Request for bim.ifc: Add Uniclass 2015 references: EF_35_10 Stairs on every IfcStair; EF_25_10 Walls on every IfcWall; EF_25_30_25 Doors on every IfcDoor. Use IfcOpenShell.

First a look at what the model holds.

```python
import ifcopenshell

model = ifcopenshell.open("bim.ifc")
print(model.schema)
print("classifications:", [c.Name for c in model.by_type("IfcClassification")])
for ifc_class in ("IfcDoor", "IfcRoof", "IfcStair", "IfcWall", "IfcWindow"):
    print(ifc_class, len(model.by_type(ifc_class)))
```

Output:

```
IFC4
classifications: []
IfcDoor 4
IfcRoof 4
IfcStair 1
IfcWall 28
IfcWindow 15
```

```python
import ifcopenshell
import ifcopenshell.api.classification

model = ifcopenshell.open("bim.ifc")

system = ifcopenshell.api.classification.add_classification(model, classification="Uniclass 2015")

codes = {
    "IfcStair": ("EF_35_10", "Stairs"),
    "IfcWall": ("EF_25_10", "Walls"),
    "IfcDoor": ("EF_25_30_25", "Doors"),
}
for ifc_class, (code, name) in codes.items():
    products = model.by_type(ifc_class)
    ifcopenshell.api.classification.add_reference(
        model, products=products, classification=system, identification=code, name=name
    )
    print(code, len(products))

model.write("bim_rev.ifc")
```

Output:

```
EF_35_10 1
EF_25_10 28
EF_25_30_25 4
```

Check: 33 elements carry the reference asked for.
